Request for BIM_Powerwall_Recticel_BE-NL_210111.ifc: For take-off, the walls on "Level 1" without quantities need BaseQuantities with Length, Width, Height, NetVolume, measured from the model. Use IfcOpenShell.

First a look at what the model holds.

```python
import ifcopenshell
import ifcopenshell.util.element
import ifcopenshell.util.unit

model = ifcopenshell.open("BIM_Powerwall_Recticel_BE-NL_210111.ifc")
print(model.schema)
for unit_type in ("LENGTHUNIT", "AREAUNIT", "VOLUMEUNIT"):
    print(unit_type, ifcopenshell.util.unit.calculate_unit_scale(model, unit_type))
storey = next(s for s in model.by_type("IfcBuildingStorey") if s.Name == "Level 1")
walls = [e for e in ifcopenshell.util.element.get_decomposition(storey) if e.is_a("IfcWall")]
for e in sorted(walls, key=lambda e: e.id()):
    print(e.id(), e.is_a(), e.Name, list(ifcopenshell.util.element.get_psets(e, qtos_only=True)), sep=" | ")
```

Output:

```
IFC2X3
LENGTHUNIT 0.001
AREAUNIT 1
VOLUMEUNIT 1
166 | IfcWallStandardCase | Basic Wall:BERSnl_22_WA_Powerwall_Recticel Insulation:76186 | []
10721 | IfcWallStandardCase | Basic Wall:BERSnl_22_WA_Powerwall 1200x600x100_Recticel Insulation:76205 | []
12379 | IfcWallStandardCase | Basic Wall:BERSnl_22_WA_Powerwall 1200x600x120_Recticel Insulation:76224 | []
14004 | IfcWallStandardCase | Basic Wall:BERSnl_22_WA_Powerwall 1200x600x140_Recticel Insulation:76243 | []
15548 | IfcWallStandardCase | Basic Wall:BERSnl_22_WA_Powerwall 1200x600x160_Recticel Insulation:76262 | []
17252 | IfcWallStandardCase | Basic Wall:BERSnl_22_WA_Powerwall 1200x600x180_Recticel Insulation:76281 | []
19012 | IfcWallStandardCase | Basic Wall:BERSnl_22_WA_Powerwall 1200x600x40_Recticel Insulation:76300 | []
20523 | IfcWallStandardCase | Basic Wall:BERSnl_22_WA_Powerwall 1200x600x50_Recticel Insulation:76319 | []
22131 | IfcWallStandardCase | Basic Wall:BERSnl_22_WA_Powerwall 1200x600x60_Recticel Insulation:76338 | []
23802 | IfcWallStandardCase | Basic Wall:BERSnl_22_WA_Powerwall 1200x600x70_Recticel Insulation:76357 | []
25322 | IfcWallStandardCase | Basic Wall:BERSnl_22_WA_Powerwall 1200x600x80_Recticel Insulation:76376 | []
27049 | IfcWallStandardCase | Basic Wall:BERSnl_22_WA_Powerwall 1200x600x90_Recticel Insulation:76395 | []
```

```python
import ifcopenshell
import ifcopenshell.api.pset
import ifcopenshell.geom
import ifcopenshell.util.element
import ifcopenshell.util.shape
import ifcopenshell.util.unit

model = ifcopenshell.open("BIM_Powerwall_Recticel_BE-NL_210111.ifc")
unit_scale = ifcopenshell.util.unit.calculate_unit_scale(model)
volume_scale = ifcopenshell.util.unit.calculate_unit_scale(model, "VOLUMEUNIT")
settings = ifcopenshell.geom.settings()

storey = next(s for s in model.by_type("IfcBuildingStorey") if s.Name == "Level 1")
walls = [e for e in ifcopenshell.util.element.get_decomposition(storey) if e.is_a("IfcWall")]

for e in sorted(walls, key=lambda e: e.id()):
    if ifcopenshell.util.element.get_psets(e, qtos_only=True, should_inherit=False):
        continue
    # Geometry comes back in metres, in the element's own axes.
    shape = ifcopenshell.geom.create_shape(settings, e)
    values = {
        "Length": ifcopenshell.util.shape.get_x(shape.geometry) / unit_scale,
        "Width": ifcopenshell.util.shape.get_y(shape.geometry) / unit_scale,
        "Height": ifcopenshell.util.shape.get_z(shape.geometry) / unit_scale,
        "NetVolume": ifcopenshell.util.shape.get_volume(shape.geometry) / volume_scale,
    }
    qto = ifcopenshell.api.pset.add_qto(model, product=e, name="BaseQuantities")
    ifcopenshell.api.pset.edit_qto(model, qto=qto, properties=values)
    print(e.id(), {k: round(v, 3) for k, v in values.items()})

model.write("BIM_Powerwall_Recticel_BE-NL_210111_updated.ifc")
```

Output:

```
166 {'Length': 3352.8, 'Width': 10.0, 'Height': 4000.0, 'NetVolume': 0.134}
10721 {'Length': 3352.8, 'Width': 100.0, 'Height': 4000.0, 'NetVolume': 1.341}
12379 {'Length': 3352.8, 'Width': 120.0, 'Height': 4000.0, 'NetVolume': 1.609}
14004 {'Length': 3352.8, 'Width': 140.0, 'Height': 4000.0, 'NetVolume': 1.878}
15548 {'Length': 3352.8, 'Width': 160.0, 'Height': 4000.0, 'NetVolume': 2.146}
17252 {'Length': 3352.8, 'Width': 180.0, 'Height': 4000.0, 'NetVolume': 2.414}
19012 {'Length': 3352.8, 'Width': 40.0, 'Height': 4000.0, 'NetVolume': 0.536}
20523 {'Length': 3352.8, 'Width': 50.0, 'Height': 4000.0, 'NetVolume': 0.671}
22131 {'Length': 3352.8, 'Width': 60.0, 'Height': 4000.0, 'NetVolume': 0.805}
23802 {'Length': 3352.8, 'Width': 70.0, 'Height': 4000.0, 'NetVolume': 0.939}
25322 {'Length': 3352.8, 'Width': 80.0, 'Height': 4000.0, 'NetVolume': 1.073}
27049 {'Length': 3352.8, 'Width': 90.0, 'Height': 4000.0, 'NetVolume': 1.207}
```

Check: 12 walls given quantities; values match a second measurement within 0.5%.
